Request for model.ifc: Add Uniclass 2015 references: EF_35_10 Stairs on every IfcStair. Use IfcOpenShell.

First a look at what the model holds.

```python
import ifcopenshell

model = ifcopenshell.open("model.ifc")
print(model.schema)
print("classifications:", [c.Name for c in model.by_type("IfcClassification")])
for ifc_class in ("IfcDoor", "IfcRoof", "IfcStair", "IfcWall", "IfcWindow"):
    print(ifc_class, len(model.by_type(ifc_class)))
```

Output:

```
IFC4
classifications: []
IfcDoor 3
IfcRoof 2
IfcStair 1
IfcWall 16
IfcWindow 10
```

```python
import ifcopenshell
import ifcopenshell.api.classification

model = ifcopenshell.open("model.ifc")

system = ifcopenshell.api.classification.add_classification(model, classification="Uniclass 2015")

codes = {
    "IfcStair": ("EF_35_10", "Stairs"),
}
for ifc_class, (code, name) in codes.items():
    products = model.by_type(ifc_class)
    ifcopenshell.api.classification.add_reference(
        model, products=products, classification=system, identification=code, name=name
    )
    print(code, len(products))

model.write("model_edited.ifc")
```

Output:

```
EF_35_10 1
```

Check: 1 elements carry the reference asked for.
